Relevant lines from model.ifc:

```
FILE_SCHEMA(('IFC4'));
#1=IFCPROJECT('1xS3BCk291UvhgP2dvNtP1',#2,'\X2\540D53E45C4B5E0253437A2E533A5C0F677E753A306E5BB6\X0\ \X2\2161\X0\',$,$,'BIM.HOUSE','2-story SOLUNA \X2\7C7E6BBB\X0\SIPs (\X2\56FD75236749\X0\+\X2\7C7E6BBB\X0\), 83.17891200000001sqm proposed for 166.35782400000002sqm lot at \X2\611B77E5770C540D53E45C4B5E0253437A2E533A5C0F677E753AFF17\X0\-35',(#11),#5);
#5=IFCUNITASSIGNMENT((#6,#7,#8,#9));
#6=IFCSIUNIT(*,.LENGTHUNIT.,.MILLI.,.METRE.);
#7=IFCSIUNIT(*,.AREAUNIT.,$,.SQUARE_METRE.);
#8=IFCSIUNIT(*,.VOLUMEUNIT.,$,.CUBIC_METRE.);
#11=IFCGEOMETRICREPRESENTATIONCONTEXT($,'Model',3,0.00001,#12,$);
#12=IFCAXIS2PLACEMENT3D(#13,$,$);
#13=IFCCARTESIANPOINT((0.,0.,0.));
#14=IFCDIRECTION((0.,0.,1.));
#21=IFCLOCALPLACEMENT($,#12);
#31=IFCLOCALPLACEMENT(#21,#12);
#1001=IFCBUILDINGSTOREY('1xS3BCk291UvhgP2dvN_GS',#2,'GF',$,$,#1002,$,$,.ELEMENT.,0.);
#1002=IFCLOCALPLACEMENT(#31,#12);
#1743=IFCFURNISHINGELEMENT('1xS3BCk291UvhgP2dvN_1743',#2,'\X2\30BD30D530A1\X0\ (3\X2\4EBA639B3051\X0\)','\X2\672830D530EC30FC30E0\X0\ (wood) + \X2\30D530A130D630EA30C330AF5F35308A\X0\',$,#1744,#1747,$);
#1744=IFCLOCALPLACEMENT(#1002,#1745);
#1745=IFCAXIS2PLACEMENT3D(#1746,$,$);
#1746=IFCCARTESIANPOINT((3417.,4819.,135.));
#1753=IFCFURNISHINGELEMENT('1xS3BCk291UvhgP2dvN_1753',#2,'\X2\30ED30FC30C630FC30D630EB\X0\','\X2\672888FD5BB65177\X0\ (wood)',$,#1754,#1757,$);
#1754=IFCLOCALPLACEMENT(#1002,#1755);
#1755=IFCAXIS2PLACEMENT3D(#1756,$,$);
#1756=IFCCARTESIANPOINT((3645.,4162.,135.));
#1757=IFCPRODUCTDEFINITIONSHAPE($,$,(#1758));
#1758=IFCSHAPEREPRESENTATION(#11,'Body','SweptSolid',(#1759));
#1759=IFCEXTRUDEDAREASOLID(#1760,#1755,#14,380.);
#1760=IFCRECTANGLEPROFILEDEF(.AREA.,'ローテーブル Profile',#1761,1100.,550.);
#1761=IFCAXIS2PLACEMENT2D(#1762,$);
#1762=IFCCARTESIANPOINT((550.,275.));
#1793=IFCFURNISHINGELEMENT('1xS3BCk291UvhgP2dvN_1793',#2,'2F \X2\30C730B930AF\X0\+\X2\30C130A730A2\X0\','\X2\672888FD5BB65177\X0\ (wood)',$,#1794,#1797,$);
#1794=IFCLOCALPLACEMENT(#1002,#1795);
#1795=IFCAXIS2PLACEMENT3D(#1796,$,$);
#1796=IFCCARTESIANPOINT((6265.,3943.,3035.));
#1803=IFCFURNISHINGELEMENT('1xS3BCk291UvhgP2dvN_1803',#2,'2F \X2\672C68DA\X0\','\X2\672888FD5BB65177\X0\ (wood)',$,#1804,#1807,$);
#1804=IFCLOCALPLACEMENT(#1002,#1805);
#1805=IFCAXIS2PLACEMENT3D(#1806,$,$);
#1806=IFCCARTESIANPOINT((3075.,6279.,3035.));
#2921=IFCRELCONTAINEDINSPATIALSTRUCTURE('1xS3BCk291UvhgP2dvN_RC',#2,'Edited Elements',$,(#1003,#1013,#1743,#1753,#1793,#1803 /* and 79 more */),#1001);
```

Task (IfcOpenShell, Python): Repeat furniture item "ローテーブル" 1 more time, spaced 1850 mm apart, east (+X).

```python
import numpy as np
import ifcopenshell
import ifcopenshell.api.geometry
import ifcopenshell.api.root
import ifcopenshell.util.element
import ifcopenshell.util.placement

model = ifcopenshell.open("model.ifc")


def reuse_history(source, copy):
    """copy_class also copies each property set's owner history, people and application; keep the originals."""
    for rel in copy.IsDefinedBy:
        if rel.is_a("IfcRelDefinesByProperties") and (history := rel.RelatingPropertyDefinition.OwnerHistory):
            rel.RelatingPropertyDefinition.OwnerHistory = source.OwnerHistory
            ifcopenshell.util.element.remove_deep2(model, history)


source = model.by_guid("1xS3BCk291UvhgP2dvN_1753")
base = ifcopenshell.util.placement.get_local_placement(source.ObjectPlacement)
step = np.array([1.0, 0.0, 0.0]) * 1850.0

for i in range(1, 2):
    copy = ifcopenshell.api.root.copy_class(model, product=source)
    copy.Representation = ifcopenshell.util.element.copy_deep(
        model, source.Representation, exclude=["IfcGeometricRepresentationContext", "IfcRepresentationMap"]
    )
    reuse_history(source, copy)
    matrix = base.copy()
    matrix[:3, 3] += i * step
    print("added at", matrix[:3, 3].round(3) + 0.0)
    ifcopenshell.api.geometry.edit_object_placement(model, product=copy, matrix=matrix, is_si=False)

model.write("model-out.ifc")
```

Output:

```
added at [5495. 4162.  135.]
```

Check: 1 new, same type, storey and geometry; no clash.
